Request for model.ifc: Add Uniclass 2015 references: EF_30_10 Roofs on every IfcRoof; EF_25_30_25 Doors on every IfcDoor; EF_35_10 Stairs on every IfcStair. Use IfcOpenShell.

First a look at what the model holds.

```python
import ifcopenshell

model = ifcopenshell.open("model.ifc")
print(model.schema)
print("classifications:", [c.Name for c in model.by_type("IfcClassification")])
for ifc_class in ("IfcDoor", "IfcRoof", "IfcStair", "IfcWall", "IfcWindow"):
    print(ifc_class, len(model.by_type(ifc_class)))
```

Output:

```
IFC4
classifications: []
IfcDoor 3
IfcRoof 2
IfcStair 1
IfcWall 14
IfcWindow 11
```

```python
import ifcopenshell
import ifcopenshell.api.classification

model = ifcopenshell.open("model.ifc")

system = ifcopenshell.api.classification.add_classification(model, classification="Uniclass 2015")

codes = {
    "IfcRoof": ("EF_30_10", "Roofs"),
    "IfcDoor": ("EF_25_30_25", "Doors"),
    "IfcStair": ("EF_35_10", "Stairs"),
}
for ifc_class, (code, name) in codes.items():
    products = model.by_type(ifc_class)
    ifcopenshell.api.classification.add_reference(
        model, products=products, classification=system, identification=code, name=name
    )
    print(code, len(products))

model.write("model_edited.ifc")
```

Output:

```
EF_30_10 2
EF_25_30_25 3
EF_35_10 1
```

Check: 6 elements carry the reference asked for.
